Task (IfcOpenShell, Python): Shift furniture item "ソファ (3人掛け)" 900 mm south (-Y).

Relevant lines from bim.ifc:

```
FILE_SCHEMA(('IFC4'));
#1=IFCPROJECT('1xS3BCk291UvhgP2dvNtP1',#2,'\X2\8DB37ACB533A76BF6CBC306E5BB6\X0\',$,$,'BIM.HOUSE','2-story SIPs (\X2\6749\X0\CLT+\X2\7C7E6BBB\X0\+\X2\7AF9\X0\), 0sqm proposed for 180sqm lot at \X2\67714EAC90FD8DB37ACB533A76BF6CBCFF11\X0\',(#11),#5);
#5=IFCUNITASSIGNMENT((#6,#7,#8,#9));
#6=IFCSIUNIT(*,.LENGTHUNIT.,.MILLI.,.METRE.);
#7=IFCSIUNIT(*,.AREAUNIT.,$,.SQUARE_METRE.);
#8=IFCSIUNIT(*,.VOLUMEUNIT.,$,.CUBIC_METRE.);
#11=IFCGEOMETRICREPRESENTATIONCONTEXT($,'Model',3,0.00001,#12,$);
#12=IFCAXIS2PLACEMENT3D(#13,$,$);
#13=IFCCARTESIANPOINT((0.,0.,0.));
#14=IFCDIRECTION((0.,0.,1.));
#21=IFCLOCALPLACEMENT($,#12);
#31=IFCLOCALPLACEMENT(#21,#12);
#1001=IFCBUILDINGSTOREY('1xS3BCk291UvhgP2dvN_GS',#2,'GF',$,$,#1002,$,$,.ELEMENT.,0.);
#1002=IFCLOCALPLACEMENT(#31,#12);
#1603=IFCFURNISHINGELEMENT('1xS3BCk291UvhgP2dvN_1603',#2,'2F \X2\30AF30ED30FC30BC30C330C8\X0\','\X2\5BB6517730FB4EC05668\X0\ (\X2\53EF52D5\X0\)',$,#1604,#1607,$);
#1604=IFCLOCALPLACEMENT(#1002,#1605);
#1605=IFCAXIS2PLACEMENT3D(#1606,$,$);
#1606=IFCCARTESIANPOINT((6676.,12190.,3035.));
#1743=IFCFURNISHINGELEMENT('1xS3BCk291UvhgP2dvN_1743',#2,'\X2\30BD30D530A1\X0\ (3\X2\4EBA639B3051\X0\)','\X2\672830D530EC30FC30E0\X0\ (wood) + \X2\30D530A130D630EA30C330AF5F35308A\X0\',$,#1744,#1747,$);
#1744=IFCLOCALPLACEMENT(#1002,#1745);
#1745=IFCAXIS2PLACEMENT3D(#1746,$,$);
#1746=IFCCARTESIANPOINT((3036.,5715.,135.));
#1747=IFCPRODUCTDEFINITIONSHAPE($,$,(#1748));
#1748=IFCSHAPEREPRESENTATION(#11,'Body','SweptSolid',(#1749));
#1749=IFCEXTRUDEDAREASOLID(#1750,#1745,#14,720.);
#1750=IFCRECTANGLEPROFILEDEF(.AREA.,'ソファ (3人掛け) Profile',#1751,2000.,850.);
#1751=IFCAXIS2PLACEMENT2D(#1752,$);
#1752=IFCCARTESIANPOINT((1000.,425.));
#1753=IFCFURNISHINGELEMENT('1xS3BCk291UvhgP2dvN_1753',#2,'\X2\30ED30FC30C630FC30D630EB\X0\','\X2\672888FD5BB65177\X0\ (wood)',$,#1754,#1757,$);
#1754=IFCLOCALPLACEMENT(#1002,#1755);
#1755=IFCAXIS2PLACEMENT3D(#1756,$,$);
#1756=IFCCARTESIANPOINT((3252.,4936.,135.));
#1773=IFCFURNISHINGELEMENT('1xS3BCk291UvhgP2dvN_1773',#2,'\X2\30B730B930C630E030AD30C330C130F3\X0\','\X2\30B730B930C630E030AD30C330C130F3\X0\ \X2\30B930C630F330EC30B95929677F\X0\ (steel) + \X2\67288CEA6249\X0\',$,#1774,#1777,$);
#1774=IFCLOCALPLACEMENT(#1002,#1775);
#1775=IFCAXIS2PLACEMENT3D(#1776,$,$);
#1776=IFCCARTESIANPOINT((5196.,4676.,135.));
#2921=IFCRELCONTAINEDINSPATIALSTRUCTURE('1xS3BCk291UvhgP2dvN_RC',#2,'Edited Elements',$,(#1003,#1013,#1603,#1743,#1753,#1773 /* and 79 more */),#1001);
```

```python
import ifcopenshell
import ifcopenshell.api.geometry
import ifcopenshell.util.placement
import ifcopenshell.util.unit

model = ifcopenshell.open("bim.ifc")
unit_scale = ifcopenshell.util.unit.calculate_unit_scale(model)

item = model.by_id(1743)
matrix = ifcopenshell.util.placement.get_local_placement(item.ObjectPlacement)
matrix[1, 3] -= 0.9 / unit_scale
ifcopenshell.api.geometry.edit_object_placement(model, product=item, matrix=matrix, is_si=False)

print(ifcopenshell.util.placement.get_local_placement(item.ObjectPlacement).round(3) + 0.0)

model.write("bim_updated.ifc")
```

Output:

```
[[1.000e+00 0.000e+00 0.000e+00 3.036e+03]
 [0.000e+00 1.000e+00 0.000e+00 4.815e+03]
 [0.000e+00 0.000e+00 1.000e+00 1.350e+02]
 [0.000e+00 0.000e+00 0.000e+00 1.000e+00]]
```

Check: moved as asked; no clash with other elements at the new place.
